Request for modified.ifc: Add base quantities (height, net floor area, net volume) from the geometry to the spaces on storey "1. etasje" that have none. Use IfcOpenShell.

First a look at what the model holds.

```python
import ifcopenshell
import ifcopenshell.util.element
import ifcopenshell.util.unit

model = ifcopenshell.open("modified.ifc")
print(model.schema)
for unit_type in ("LENGTHUNIT", "AREAUNIT", "VOLUMEUNIT"):
    print(unit_type, ifcopenshell.util.unit.calculate_unit_scale(model, unit_type))
storey = next(s for s in model.by_type("IfcBuildingStorey") if s.Name == "1. etasje")
spaces = [e for e in ifcopenshell.util.element.get_decomposition(storey) if e.is_a("IfcSpace")]
for e in sorted(spaces, key=lambda e: e.id()):
    print(e.id(), e.is_a(), e.Name, list(ifcopenshell.util.element.get_psets(e, qtos_only=True)), sep=" | ")
```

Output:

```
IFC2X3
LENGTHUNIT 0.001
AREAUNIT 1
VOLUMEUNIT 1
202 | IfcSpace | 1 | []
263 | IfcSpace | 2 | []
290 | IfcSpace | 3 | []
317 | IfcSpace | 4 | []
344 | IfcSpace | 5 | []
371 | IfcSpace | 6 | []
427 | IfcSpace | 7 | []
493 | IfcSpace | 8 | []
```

```python
import ifcopenshell
import ifcopenshell.api.pset
import ifcopenshell.geom
import ifcopenshell.util.element
import ifcopenshell.util.shape
import ifcopenshell.util.unit

model = ifcopenshell.open("modified.ifc")
unit_scale = ifcopenshell.util.unit.calculate_unit_scale(model)
area_scale = ifcopenshell.util.unit.calculate_unit_scale(model, "AREAUNIT")
volume_scale = ifcopenshell.util.unit.calculate_unit_scale(model, "VOLUMEUNIT")
settings = ifcopenshell.geom.settings()

storey = next(s for s in model.by_type("IfcBuildingStorey") if s.Name == "1. etasje")
spaces = [e for e in ifcopenshell.util.element.get_decomposition(storey) if e.is_a("IfcSpace")]

for e in sorted(spaces, key=lambda e: e.id()):
    if ifcopenshell.util.element.get_psets(e, qtos_only=True, should_inherit=False):
        continue
    # Geometry comes back in metres, in the element's own axes.
    shape = ifcopenshell.geom.create_shape(settings, e)
    values = {
        "Height": ifcopenshell.util.shape.get_z(shape.geometry) / unit_scale,
        "NetFloorArea": ifcopenshell.util.shape.get_footprint_area(shape.geometry) / area_scale,
        "NetVolume": ifcopenshell.util.shape.get_volume(shape.geometry) / volume_scale,
    }
    qto = ifcopenshell.api.pset.add_qto(model, product=e, name="BaseQuantities")
    ifcopenshell.api.pset.edit_qto(model, qto=qto, properties=values)
    print(e.id(), {k: round(v, 3) for k, v in values.items()})

model.write("modified_rev.ifc")
```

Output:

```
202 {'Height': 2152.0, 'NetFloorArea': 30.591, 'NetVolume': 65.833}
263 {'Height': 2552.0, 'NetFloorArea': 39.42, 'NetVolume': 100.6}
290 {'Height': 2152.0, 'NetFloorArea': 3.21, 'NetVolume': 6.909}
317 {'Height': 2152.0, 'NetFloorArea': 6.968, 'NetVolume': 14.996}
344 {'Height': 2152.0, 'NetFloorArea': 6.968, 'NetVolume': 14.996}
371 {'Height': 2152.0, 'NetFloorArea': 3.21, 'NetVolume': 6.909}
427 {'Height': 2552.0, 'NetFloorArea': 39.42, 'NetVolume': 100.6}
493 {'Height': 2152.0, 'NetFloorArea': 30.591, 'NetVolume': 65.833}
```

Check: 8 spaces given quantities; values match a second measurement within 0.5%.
